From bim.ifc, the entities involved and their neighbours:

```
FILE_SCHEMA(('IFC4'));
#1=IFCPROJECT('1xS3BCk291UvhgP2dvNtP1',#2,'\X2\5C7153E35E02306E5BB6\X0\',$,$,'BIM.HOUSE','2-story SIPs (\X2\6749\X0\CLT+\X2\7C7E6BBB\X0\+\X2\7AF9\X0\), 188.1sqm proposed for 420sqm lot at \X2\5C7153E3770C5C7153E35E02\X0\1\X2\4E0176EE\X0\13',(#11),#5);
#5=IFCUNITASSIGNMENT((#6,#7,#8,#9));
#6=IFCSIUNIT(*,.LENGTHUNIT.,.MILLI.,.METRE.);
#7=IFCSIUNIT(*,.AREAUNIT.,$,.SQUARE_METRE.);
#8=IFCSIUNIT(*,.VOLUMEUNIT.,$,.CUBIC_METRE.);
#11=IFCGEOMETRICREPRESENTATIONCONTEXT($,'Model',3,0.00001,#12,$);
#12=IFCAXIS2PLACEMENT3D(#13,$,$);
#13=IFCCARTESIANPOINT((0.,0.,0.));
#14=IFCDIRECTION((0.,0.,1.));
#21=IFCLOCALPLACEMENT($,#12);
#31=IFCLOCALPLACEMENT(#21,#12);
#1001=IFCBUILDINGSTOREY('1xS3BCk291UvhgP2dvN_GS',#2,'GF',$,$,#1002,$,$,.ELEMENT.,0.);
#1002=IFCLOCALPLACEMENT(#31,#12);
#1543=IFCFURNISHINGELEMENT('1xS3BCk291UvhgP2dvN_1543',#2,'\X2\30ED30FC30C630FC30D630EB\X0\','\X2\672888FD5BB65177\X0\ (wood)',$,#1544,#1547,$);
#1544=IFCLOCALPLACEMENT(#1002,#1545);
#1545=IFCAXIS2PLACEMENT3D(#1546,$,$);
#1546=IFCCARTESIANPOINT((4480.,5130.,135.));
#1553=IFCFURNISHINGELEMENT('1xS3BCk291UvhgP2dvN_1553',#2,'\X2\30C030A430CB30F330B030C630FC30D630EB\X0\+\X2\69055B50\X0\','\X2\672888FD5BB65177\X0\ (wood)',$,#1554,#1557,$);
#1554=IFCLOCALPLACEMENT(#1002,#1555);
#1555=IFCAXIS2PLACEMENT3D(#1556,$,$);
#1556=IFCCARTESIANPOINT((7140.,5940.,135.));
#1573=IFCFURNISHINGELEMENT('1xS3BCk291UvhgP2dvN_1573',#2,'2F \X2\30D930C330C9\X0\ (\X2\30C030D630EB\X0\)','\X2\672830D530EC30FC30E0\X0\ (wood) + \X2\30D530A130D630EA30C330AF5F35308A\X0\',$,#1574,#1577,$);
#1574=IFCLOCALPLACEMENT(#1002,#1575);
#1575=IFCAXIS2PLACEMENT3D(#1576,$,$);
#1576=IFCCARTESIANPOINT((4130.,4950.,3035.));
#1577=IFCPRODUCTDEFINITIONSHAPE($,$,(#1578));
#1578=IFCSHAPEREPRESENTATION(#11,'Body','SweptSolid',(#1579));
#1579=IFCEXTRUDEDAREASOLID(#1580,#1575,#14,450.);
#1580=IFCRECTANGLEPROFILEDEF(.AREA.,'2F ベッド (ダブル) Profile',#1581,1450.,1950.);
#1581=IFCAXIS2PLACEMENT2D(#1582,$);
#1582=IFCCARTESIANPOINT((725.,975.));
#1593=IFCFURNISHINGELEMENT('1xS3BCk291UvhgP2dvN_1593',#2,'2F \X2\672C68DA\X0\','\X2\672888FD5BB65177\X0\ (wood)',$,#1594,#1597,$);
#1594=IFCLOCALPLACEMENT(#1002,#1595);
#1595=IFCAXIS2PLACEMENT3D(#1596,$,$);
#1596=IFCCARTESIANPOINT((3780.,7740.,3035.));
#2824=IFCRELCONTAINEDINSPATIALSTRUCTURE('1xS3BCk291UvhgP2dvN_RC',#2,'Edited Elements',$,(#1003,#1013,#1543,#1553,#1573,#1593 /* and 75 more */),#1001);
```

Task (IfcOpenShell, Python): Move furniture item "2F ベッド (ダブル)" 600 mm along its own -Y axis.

```python
import ifcopenshell
import ifcopenshell.api.geometry
import ifcopenshell.util.placement
import ifcopenshell.util.unit

model = ifcopenshell.open("bim.ifc")
unit_scale = ifcopenshell.util.unit.calculate_unit_scale(model)

item = model.by_guid("1xS3BCk291UvhgP2dvN_1573")
matrix = ifcopenshell.util.placement.get_local_placement(item.ObjectPlacement)
matrix[:3, 3] -= matrix[:3, 1] * 0.6 / unit_scale
ifcopenshell.api.geometry.edit_object_placement(model, product=item, matrix=matrix, is_si=False)

print(ifcopenshell.util.placement.get_local_placement(item.ObjectPlacement).round(3) + 0.0)

model.write("bim_rev.ifc")
```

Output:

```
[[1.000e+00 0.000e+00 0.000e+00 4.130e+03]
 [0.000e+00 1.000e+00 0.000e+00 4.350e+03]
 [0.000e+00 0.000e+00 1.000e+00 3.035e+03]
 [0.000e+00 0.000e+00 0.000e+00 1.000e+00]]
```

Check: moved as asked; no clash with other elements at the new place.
